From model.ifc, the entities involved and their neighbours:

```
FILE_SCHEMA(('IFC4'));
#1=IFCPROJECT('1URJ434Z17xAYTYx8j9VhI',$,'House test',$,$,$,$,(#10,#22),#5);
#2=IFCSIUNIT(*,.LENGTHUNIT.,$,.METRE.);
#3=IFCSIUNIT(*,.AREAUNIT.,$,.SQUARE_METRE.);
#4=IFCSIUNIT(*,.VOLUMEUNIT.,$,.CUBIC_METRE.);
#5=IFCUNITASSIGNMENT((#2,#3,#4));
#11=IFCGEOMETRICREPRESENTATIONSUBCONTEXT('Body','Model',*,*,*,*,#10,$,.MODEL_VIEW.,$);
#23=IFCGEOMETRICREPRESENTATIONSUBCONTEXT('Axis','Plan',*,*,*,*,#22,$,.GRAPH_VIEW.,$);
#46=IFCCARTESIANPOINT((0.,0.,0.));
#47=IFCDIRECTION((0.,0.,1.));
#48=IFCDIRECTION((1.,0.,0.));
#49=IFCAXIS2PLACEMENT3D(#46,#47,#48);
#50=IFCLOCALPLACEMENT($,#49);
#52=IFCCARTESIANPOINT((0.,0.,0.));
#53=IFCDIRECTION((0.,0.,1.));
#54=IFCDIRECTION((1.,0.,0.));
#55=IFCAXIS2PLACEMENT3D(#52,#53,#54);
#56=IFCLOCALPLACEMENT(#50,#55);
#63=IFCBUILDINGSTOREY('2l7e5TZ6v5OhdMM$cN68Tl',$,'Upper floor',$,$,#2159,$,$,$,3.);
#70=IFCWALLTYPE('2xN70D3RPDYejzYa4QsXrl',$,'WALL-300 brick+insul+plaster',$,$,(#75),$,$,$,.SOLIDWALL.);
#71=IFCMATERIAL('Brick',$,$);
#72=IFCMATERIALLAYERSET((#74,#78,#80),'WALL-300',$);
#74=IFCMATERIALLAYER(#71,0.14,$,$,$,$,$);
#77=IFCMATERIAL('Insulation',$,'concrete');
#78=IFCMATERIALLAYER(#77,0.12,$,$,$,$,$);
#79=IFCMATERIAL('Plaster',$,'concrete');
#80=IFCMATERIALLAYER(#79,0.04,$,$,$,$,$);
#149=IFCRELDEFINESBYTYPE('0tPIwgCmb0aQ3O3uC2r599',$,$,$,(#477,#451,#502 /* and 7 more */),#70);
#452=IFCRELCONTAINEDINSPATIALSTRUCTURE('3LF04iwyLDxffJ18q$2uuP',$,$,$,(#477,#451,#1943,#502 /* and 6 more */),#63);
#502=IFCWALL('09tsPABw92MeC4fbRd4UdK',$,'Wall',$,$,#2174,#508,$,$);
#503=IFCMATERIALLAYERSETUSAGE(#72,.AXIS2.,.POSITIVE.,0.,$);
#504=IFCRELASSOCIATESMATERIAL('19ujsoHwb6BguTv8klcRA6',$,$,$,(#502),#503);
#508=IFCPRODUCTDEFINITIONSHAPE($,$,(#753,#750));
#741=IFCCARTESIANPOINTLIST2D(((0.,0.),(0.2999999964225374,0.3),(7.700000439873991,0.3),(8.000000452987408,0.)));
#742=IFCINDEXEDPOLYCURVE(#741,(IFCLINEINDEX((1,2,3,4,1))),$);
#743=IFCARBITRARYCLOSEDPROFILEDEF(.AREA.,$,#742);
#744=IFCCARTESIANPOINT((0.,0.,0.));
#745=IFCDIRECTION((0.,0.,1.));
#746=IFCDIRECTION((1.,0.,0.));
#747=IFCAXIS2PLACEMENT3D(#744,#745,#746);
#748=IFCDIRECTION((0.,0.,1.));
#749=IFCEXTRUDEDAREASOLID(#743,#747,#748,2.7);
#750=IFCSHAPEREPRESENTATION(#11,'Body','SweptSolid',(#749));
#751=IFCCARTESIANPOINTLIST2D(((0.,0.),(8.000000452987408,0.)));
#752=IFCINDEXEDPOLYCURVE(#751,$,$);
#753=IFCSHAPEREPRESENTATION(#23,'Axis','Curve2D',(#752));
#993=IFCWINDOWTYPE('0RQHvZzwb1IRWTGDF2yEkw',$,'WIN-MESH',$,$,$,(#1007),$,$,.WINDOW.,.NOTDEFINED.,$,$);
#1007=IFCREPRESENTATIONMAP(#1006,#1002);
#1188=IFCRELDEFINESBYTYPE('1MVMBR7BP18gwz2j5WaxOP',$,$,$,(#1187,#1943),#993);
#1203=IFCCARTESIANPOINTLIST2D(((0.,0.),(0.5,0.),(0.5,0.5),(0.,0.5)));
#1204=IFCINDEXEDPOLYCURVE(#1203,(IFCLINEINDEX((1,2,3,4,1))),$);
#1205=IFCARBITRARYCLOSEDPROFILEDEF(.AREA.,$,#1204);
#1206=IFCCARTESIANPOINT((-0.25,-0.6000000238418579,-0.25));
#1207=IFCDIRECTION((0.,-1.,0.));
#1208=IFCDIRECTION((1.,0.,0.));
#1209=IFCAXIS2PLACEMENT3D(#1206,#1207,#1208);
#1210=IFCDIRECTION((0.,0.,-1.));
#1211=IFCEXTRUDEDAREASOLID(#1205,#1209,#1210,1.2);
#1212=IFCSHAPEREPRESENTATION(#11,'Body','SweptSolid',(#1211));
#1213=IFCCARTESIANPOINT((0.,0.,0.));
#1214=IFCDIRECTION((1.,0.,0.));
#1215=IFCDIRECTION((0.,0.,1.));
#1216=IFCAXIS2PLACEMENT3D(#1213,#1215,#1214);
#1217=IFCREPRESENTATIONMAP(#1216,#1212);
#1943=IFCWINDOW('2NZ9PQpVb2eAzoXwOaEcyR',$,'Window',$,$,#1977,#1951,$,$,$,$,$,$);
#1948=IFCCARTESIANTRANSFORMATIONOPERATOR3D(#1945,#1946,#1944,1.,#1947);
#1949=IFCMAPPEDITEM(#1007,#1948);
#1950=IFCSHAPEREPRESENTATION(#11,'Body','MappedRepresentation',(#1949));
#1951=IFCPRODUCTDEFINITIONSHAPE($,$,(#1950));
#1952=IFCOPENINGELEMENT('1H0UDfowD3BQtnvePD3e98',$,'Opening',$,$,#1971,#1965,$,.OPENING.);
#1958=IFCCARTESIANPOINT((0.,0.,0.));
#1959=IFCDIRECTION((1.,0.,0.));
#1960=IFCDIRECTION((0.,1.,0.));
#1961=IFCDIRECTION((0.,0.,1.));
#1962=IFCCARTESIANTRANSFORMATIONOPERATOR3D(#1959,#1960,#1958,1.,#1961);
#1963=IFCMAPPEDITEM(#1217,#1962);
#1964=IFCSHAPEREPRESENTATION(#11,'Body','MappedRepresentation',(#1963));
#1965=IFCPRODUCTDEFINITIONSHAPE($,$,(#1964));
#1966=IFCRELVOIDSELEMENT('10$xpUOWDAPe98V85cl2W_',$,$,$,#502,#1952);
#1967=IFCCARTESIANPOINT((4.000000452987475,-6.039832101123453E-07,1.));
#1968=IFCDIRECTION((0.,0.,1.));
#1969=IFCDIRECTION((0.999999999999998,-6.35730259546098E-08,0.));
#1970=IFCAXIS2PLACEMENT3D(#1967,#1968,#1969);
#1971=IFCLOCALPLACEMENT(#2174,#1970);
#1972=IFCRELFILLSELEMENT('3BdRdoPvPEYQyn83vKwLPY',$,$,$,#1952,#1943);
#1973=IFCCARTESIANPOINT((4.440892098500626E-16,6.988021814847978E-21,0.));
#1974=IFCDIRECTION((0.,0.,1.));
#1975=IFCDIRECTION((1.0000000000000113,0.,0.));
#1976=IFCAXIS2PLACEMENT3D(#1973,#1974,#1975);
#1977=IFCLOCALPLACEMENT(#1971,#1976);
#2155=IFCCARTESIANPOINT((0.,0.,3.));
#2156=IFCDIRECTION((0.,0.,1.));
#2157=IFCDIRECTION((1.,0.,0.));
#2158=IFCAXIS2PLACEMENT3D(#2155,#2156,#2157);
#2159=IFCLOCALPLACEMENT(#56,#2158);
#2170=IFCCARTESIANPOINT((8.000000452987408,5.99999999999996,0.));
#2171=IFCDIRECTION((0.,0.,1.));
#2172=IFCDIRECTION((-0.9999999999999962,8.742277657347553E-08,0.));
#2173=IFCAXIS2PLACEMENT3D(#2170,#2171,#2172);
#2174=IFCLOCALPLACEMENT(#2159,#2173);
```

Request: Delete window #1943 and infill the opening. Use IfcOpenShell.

```python
import ifcopenshell
import ifcopenshell.api.feature
import ifcopenshell.api.root
import ifcopenshell.geom
import ifcopenshell.util.shape

model = ifcopenshell.open("model.ifc")
settings = ifcopenshell.geom.settings()


def volume(element):
    """Net volume in cubic metres, openings subtracted."""
    shape = ifcopenshell.geom.create_shape(settings, element)
    return ifcopenshell.util.shape.get_volume(shape.geometry)


window = model.by_id(1943)
opening = window.FillsVoids[0].RelatingOpeningElement
wall = opening.VoidsElements[0].RelatingBuildingElement
before = volume(wall)

ifcopenshell.api.root.remove_product(model, product=window)
ifcopenshell.api.feature.remove_feature(model, feature=opening)

after = volume(wall)

print(f"wall volume {before:.3f} -> {after:.3f} m3")

model.write("model_updated.ifc")
```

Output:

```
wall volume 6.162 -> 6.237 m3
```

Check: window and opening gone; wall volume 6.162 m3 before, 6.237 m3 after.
